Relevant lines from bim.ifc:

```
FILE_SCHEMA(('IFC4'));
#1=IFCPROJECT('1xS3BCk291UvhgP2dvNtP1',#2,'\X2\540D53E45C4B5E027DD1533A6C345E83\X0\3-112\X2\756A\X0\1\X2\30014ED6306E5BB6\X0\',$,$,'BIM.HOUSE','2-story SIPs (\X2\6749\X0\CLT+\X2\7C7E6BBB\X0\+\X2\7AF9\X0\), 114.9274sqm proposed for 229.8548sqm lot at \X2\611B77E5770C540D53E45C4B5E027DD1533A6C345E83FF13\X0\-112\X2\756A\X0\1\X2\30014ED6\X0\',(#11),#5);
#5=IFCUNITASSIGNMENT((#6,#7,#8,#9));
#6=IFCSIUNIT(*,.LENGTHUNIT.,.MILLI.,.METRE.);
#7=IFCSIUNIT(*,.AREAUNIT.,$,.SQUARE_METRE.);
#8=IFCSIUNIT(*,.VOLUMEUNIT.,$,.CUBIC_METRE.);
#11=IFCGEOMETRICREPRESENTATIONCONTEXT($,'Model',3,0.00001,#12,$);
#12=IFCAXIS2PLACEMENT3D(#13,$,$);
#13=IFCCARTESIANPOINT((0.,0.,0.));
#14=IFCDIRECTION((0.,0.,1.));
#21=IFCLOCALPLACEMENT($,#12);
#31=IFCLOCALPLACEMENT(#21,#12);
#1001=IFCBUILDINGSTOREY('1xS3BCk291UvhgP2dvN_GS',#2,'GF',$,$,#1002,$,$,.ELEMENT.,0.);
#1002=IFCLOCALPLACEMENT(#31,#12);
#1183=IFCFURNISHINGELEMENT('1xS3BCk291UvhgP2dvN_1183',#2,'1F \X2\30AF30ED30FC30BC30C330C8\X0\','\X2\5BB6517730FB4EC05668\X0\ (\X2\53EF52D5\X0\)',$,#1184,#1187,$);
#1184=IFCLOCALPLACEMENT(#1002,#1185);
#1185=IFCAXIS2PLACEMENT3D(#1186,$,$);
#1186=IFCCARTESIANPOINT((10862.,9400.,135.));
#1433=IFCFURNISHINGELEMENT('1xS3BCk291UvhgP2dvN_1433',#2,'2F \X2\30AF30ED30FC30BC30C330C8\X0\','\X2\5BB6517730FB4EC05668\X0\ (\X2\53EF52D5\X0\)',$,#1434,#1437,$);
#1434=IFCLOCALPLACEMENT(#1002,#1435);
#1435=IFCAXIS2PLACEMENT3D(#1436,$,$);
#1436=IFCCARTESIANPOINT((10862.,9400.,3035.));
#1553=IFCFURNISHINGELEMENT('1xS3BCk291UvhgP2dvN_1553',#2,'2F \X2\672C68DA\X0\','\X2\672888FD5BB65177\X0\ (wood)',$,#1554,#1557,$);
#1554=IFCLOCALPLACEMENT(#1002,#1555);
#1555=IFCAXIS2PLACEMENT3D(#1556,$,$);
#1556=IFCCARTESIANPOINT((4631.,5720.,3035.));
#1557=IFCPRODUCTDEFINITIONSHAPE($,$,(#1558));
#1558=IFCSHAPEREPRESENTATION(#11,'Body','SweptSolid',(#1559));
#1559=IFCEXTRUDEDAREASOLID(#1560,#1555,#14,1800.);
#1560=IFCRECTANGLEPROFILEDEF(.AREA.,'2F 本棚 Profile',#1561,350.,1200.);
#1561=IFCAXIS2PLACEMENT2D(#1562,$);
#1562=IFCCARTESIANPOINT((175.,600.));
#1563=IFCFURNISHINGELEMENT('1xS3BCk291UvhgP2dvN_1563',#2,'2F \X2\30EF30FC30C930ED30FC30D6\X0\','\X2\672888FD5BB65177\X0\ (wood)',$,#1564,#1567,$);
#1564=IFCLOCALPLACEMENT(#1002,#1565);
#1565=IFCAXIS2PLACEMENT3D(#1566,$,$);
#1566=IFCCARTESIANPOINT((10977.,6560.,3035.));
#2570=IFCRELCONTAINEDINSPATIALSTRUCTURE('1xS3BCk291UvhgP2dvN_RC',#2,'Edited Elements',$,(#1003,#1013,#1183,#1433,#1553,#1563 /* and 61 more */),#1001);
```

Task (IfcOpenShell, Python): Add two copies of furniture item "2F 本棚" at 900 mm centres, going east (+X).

```python
import numpy as np
import ifcopenshell
import ifcopenshell.api.geometry
import ifcopenshell.api.root
import ifcopenshell.util.element
import ifcopenshell.util.placement
import ifcopenshell.util.unit

model = ifcopenshell.open("bim.ifc")
unit_scale = ifcopenshell.util.unit.calculate_unit_scale(model)


def reuse_history(source, copy):
    """copy_class also copies each property set's owner history, people and application; keep the originals."""
    for rel in copy.IsDefinedBy:
        if rel.is_a("IfcRelDefinesByProperties") and (history := rel.RelatingPropertyDefinition.OwnerHistory):
            rel.RelatingPropertyDefinition.OwnerHistory = source.OwnerHistory
            ifcopenshell.util.element.remove_deep2(model, history)


source = model.by_id(1553)
base = ifcopenshell.util.placement.get_local_placement(source.ObjectPlacement)
step = np.array([1.0, 0.0, 0.0]) * 0.9 / unit_scale

for i in range(1, 3):
    copy = ifcopenshell.api.root.copy_class(model, product=source)
    copy.Representation = ifcopenshell.util.element.copy_deep(
        model, source.Representation, exclude=["IfcGeometricRepresentationContext", "IfcRepresentationMap"]
    )
    reuse_history(source, copy)
    matrix = base.copy()
    matrix[:3, 3] += i * step
    print("added at", matrix[:3, 3].round(3) + 0.0)
    ifcopenshell.api.geometry.edit_object_placement(model, product=copy, matrix=matrix, is_si=False)

model.write("bim-out.ifc")
```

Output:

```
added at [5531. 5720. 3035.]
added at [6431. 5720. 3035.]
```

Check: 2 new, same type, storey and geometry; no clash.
